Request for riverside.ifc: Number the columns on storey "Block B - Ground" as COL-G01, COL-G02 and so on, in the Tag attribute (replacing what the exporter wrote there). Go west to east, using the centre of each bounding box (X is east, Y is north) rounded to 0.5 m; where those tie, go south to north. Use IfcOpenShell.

First a look at what the model holds.

```python
import ifcopenshell
import ifcopenshell.util.element
import ifcopenshell.util.placement

model = ifcopenshell.open("riverside.ifc")
print(model.schema)
storey = next(s for s in model.by_type("IfcBuildingStorey") if s.Name == "Block B - Ground")
columns = [e for e in ifcopenshell.util.element.get_decomposition(storey) if e.is_a("IfcColumn")]
for e in sorted(columns, key=lambda e: e.id()):
    origin = ifcopenshell.util.placement.get_local_placement(e.ObjectPlacement)[:3, 3]
    print(e.id(), e.Tag, e.Name, origin.round(2) + 0.0, sep=" | ")
```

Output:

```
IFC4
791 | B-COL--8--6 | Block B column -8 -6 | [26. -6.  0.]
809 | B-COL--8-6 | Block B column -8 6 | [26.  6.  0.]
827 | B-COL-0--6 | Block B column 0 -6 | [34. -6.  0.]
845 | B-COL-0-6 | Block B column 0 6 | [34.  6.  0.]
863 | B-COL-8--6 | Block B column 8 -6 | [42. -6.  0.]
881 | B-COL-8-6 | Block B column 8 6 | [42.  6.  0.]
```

```python
import ifcopenshell
import ifcopenshell.geom
import ifcopenshell.util.element
import ifcopenshell.util.shape

model = ifcopenshell.open("riverside.ifc")
settings = ifcopenshell.geom.settings()
settings.set("use-world-coords", True)


def centre(element):
    shape = ifcopenshell.geom.create_shape(settings, element)
    return ifcopenshell.util.shape.get_bbox_centroid(shape.geometry)


storey = next(s for s in model.by_type("IfcBuildingStorey") if s.Name == "Block B - Ground")
columns = [e for e in ifcopenshell.util.element.get_decomposition(storey) if e.is_a("IfcColumn")]

# Insertion points can sit at a corner or the storey origin, so sort by the geometry (in metres).
centres = {e: centre(e) for e in columns}
columns.sort(key=lambda e: (round(centres[e][0] / 0.5), centres[e][1]))

for i, e in enumerate(columns, start=1):
    number = f"COL-G{i:02d}"
    e.Tag = number
    print(e.id(), number)

model.write("riverside-out.ifc")
```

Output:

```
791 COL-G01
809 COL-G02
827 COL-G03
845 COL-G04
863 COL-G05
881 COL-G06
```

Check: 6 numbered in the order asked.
